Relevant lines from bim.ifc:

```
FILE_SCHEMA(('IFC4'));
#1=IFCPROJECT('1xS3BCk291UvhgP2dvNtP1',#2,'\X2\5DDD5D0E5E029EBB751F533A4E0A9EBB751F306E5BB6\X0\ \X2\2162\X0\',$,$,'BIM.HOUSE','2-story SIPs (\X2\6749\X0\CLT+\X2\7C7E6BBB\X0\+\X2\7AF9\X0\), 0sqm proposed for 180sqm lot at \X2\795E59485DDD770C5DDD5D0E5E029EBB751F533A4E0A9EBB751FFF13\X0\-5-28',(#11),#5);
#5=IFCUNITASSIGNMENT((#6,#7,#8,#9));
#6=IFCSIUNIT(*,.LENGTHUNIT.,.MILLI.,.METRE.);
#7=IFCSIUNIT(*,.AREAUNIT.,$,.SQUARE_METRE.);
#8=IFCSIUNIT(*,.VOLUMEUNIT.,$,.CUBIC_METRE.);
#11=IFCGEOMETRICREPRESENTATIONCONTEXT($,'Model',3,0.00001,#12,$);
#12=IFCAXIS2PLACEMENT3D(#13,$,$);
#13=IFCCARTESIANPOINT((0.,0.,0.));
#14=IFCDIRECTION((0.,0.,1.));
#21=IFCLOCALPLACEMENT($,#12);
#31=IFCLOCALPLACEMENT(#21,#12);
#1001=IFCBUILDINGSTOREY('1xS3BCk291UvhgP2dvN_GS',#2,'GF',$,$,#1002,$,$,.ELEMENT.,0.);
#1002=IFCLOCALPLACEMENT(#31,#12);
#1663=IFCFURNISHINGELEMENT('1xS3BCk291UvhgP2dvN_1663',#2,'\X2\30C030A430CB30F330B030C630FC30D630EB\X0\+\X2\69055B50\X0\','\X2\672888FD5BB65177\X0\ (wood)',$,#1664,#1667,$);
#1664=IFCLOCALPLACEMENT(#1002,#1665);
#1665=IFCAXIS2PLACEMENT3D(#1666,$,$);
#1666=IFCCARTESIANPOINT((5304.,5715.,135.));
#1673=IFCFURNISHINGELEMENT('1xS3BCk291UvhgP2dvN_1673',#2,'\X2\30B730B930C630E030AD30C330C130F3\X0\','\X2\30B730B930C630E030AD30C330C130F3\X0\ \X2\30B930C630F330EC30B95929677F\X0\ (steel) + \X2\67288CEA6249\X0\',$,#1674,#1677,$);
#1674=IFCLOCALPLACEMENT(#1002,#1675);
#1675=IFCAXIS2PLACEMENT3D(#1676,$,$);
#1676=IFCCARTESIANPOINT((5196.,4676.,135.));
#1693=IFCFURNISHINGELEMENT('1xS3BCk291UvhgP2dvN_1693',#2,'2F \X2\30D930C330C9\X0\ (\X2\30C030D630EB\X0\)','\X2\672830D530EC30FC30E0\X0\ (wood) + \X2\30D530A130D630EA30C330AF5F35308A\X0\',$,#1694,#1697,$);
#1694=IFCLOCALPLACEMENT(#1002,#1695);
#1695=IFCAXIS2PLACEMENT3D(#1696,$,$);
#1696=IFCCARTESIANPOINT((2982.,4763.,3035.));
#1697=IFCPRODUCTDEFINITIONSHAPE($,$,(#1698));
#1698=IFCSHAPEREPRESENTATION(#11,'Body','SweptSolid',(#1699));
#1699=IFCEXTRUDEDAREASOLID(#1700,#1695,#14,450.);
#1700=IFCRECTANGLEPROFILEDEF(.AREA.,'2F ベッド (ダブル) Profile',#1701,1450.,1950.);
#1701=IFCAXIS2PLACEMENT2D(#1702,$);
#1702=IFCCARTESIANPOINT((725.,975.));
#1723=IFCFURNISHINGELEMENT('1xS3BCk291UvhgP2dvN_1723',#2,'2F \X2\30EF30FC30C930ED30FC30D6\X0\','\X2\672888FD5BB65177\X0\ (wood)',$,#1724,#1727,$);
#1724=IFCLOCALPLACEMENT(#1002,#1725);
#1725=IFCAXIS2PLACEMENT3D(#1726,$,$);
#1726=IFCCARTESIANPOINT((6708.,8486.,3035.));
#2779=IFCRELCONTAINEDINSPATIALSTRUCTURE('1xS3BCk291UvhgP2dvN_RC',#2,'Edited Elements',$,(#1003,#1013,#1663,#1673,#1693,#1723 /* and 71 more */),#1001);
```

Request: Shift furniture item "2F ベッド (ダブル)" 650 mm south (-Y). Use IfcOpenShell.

```python
import ifcopenshell
import ifcopenshell.api.geometry
import ifcopenshell.util.placement
import ifcopenshell.util.unit

model = ifcopenshell.open("bim.ifc")
unit_scale = ifcopenshell.util.unit.calculate_unit_scale(model)

item = model.by_id(1693)
matrix = ifcopenshell.util.placement.get_local_placement(item.ObjectPlacement)
matrix[1, 3] -= 0.65 / unit_scale
ifcopenshell.api.geometry.edit_object_placement(model, product=item, matrix=matrix, is_si=False)

print(ifcopenshell.util.placement.get_local_placement(item.ObjectPlacement).round(3) + 0.0)

model.write("bim_edited.ifc")
```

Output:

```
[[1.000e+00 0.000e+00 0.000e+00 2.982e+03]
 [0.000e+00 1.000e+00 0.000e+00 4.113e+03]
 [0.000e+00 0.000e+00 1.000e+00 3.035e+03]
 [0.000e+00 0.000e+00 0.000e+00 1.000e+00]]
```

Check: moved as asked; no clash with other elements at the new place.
